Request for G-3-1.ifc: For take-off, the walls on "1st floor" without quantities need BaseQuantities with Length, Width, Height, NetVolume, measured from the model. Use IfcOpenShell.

First a look at what the model holds.

```python
import ifcopenshell
import ifcopenshell.util.element
import ifcopenshell.util.unit

model = ifcopenshell.open("G-3-1.ifc")
print(model.schema)
for unit_type in ("LENGTHUNIT", "AREAUNIT", "VOLUMEUNIT"):
    print(unit_type, ifcopenshell.util.unit.calculate_unit_scale(model, unit_type))
storey = next(s for s in model.by_type("IfcBuildingStorey") if s.Name == "1st floor")
walls = [e for e in ifcopenshell.util.element.get_decomposition(storey) if e.is_a("IfcWall")]
for e in sorted(walls, key=lambda e: e.id()):
    print(e.id(), e.is_a(), e.Name, list(ifcopenshell.util.element.get_psets(e, qtos_only=True)), sep=" | ")
```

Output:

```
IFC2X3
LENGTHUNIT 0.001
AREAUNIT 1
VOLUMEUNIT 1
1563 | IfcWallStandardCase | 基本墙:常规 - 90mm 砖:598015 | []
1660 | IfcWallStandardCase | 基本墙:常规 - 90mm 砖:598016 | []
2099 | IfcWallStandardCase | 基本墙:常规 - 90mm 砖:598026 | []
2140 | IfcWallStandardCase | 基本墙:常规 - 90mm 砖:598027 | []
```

```python
import ifcopenshell
import ifcopenshell.api.pset
import ifcopenshell.geom
import ifcopenshell.util.element
import ifcopenshell.util.shape
import ifcopenshell.util.unit

model = ifcopenshell.open("G-3-1.ifc")
unit_scale = ifcopenshell.util.unit.calculate_unit_scale(model)
volume_scale = ifcopenshell.util.unit.calculate_unit_scale(model, "VOLUMEUNIT")
settings = ifcopenshell.geom.settings()

storey = next(s for s in model.by_type("IfcBuildingStorey") if s.Name == "1st floor")
walls = [e for e in ifcopenshell.util.element.get_decomposition(storey) if e.is_a("IfcWall")]

for e in sorted(walls, key=lambda e: e.id()):
    if ifcopenshell.util.element.get_psets(e, qtos_only=True, should_inherit=False):
        continue
    # Geometry comes back in metres, in the element's own axes.
    shape = ifcopenshell.geom.create_shape(settings, e)
    values = {
        "Length": ifcopenshell.util.shape.get_x(shape.geometry) / unit_scale,
        "Width": ifcopenshell.util.shape.get_y(shape.geometry) / unit_scale,
        "Height": ifcopenshell.util.shape.get_z(shape.geometry) / unit_scale,
        "NetVolume": ifcopenshell.util.shape.get_volume(shape.geometry) / volume_scale,
    }
    qto = ifcopenshell.api.pset.add_qto(model, product=e, name="BaseQuantities")
    ifcopenshell.api.pset.edit_qto(model, qto=qto, properties=values)
    print(e.id(), {k: round(v, 3) for k, v in values.items()})

model.write("G-3-1_updated.ifc")
```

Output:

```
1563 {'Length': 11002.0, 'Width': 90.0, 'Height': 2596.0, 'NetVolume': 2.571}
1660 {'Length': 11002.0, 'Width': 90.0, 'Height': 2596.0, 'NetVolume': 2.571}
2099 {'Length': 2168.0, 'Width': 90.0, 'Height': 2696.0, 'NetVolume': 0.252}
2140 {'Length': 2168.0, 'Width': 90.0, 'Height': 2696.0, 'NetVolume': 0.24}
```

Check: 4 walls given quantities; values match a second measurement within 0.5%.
